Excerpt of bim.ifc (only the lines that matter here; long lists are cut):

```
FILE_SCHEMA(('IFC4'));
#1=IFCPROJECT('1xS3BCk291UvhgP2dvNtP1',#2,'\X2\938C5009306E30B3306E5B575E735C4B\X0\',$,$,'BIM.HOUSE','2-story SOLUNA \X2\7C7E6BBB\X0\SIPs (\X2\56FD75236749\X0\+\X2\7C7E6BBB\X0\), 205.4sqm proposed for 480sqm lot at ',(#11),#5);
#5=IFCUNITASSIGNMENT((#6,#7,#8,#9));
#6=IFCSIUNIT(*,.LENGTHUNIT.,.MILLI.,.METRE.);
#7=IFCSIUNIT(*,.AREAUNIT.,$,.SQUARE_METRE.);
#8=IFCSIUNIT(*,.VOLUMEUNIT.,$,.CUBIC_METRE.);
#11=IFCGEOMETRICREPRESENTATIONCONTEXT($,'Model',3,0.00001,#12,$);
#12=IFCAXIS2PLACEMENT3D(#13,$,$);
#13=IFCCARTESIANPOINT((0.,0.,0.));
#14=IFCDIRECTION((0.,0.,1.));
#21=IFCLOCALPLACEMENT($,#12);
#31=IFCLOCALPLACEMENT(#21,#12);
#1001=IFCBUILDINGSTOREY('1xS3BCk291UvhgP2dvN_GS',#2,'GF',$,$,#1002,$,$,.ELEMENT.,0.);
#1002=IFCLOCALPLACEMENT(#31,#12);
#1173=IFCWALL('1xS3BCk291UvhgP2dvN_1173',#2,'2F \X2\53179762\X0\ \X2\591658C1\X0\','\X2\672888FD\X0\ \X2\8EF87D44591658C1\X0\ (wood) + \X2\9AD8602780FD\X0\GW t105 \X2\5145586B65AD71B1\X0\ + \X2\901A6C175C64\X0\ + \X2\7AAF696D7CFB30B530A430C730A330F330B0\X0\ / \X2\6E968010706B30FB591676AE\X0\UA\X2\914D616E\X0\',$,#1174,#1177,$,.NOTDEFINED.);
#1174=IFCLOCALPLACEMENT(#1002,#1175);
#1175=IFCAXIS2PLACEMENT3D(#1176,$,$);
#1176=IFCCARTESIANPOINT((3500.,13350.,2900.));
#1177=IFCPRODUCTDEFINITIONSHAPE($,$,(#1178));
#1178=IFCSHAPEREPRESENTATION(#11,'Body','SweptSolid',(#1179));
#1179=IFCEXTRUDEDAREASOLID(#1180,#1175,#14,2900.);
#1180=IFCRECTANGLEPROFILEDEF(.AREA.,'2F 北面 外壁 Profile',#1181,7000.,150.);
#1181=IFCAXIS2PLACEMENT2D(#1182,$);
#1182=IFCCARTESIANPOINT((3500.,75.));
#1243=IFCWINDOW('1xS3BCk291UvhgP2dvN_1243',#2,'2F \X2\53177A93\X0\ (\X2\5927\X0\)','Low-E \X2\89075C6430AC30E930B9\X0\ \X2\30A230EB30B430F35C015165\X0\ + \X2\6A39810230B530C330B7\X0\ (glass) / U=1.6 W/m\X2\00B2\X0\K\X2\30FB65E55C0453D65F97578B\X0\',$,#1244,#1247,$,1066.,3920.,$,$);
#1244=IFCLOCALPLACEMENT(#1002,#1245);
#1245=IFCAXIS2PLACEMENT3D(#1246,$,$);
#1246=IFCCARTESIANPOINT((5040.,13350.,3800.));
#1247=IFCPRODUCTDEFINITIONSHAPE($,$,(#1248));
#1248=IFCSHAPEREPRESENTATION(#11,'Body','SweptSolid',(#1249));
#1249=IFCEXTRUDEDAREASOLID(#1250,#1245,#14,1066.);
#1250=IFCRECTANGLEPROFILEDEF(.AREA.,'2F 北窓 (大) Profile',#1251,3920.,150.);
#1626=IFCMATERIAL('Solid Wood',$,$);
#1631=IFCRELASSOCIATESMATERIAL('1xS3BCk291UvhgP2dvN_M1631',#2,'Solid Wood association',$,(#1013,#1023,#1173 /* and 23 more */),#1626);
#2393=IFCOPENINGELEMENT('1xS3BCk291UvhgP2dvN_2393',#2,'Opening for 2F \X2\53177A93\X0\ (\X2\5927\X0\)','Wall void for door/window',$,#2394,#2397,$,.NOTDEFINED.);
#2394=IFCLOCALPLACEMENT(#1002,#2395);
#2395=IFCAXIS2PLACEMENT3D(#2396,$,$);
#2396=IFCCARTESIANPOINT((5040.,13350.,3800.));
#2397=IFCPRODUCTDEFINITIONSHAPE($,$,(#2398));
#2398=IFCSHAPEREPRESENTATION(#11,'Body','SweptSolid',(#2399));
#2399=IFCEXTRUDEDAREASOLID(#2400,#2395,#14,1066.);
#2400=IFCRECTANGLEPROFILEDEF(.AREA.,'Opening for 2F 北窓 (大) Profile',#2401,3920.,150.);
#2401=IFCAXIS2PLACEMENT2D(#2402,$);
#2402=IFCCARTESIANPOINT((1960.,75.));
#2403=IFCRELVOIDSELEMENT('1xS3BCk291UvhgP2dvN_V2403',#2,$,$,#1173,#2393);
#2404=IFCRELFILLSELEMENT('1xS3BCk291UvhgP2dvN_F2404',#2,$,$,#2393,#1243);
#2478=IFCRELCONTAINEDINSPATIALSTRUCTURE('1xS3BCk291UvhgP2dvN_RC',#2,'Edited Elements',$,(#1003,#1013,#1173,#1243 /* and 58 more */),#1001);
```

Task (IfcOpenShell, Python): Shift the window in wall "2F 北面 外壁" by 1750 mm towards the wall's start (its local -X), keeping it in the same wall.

```python
import ifcopenshell
import ifcopenshell.api.geometry
import ifcopenshell.util.placement
import ifcopenshell.util.unit

model = ifcopenshell.open("bim.ifc")
unit_scale = ifcopenshell.util.unit.calculate_unit_scale(model)

window = model.by_guid("1xS3BCk291UvhgP2dvN_1243")
opening = window.FillsVoids[0].RelatingOpeningElement
wall = opening.VoidsElements[0].RelatingBuildingElement

wall_matrix = ifcopenshell.util.placement.get_local_placement(wall.ObjectPlacement)
shift = wall_matrix[:3, 0] * -1.75 / unit_scale
before = ifcopenshell.util.placement.get_local_placement(window.ObjectPlacement)[:3, 3].copy()

# The window is not placed relative to its opening, so move both.
for product in (opening, window):
    matrix = ifcopenshell.util.placement.get_local_placement(product.ObjectPlacement)
    matrix[:3, 3] += shift
    ifcopenshell.api.geometry.edit_object_placement(model, product=product, matrix=matrix, is_si=False)

after = ifcopenshell.util.placement.get_local_placement(window.ObjectPlacement)[:3, 3]
print("window moved by", (after - before).round(3) + 0.0)

model.write("bim_v2.ifc")
```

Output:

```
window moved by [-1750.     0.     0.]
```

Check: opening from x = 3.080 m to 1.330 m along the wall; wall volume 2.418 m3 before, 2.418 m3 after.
